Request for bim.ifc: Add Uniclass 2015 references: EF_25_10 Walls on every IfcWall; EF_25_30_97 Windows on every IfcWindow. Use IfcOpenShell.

First a look at what the model holds.

```python
import ifcopenshell

model = ifcopenshell.open("bim.ifc")
print(model.schema)
print("classifications:", [c.Name for c in model.by_type("IfcClassification")])
for ifc_class in ("IfcDoor", "IfcRoof", "IfcStair", "IfcWall", "IfcWindow"):
    print(ifc_class, len(model.by_type(ifc_class)))
```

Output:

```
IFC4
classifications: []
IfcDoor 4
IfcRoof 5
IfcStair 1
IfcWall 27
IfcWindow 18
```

```python
import ifcopenshell
import ifcopenshell.api.classification

model = ifcopenshell.open("bim.ifc")

system = ifcopenshell.api.classification.add_classification(model, classification="Uniclass 2015")

codes = {
    "IfcWall": ("EF_25_10", "Walls"),
    "IfcWindow": ("EF_25_30_97", "Windows"),
}
for ifc_class, (code, name) in codes.items():
    products = model.by_type(ifc_class)
    ifcopenshell.api.classification.add_reference(
        model, products=products, classification=system, identification=code, name=name
    )
    print(code, len(products))

model.write("bim_edited.ifc")
```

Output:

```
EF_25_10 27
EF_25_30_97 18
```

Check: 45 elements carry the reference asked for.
